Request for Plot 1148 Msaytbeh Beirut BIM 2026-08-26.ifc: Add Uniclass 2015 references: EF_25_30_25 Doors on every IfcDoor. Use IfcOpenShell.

First a look at what the model holds.

```python
import ifcopenshell

model = ifcopenshell.open("Plot 1148 Msaytbeh Beirut BIM 2026-08-26.ifc")
print(model.schema)
print("classifications:", [c.Name for c in model.by_type("IfcClassification")])
for ifc_class in ("IfcDoor", "IfcRoof", "IfcStair", "IfcWall", "IfcWindow"):
    print(ifc_class, len(model.by_type(ifc_class)))
```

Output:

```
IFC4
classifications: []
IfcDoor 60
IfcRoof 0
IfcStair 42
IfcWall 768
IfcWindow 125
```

```python
import ifcopenshell
import ifcopenshell.api.classification

model = ifcopenshell.open("Plot 1148 Msaytbeh Beirut BIM 2026-08-26.ifc")

system = ifcopenshell.api.classification.add_classification(model, classification="Uniclass 2015")

codes = {
    "IfcDoor": ("EF_25_30_25", "Doors"),
}
for ifc_class, (code, name) in codes.items():
    products = model.by_type(ifc_class)
    ifcopenshell.api.classification.add_reference(
        model, products=products, classification=system, identification=code, name=name
    )
    print(code, len(products))

model.write("Plot 1148 Msaytbeh Beirut BIM 2026-08-26_v2.ifc")
```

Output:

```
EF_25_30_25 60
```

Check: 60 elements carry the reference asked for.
